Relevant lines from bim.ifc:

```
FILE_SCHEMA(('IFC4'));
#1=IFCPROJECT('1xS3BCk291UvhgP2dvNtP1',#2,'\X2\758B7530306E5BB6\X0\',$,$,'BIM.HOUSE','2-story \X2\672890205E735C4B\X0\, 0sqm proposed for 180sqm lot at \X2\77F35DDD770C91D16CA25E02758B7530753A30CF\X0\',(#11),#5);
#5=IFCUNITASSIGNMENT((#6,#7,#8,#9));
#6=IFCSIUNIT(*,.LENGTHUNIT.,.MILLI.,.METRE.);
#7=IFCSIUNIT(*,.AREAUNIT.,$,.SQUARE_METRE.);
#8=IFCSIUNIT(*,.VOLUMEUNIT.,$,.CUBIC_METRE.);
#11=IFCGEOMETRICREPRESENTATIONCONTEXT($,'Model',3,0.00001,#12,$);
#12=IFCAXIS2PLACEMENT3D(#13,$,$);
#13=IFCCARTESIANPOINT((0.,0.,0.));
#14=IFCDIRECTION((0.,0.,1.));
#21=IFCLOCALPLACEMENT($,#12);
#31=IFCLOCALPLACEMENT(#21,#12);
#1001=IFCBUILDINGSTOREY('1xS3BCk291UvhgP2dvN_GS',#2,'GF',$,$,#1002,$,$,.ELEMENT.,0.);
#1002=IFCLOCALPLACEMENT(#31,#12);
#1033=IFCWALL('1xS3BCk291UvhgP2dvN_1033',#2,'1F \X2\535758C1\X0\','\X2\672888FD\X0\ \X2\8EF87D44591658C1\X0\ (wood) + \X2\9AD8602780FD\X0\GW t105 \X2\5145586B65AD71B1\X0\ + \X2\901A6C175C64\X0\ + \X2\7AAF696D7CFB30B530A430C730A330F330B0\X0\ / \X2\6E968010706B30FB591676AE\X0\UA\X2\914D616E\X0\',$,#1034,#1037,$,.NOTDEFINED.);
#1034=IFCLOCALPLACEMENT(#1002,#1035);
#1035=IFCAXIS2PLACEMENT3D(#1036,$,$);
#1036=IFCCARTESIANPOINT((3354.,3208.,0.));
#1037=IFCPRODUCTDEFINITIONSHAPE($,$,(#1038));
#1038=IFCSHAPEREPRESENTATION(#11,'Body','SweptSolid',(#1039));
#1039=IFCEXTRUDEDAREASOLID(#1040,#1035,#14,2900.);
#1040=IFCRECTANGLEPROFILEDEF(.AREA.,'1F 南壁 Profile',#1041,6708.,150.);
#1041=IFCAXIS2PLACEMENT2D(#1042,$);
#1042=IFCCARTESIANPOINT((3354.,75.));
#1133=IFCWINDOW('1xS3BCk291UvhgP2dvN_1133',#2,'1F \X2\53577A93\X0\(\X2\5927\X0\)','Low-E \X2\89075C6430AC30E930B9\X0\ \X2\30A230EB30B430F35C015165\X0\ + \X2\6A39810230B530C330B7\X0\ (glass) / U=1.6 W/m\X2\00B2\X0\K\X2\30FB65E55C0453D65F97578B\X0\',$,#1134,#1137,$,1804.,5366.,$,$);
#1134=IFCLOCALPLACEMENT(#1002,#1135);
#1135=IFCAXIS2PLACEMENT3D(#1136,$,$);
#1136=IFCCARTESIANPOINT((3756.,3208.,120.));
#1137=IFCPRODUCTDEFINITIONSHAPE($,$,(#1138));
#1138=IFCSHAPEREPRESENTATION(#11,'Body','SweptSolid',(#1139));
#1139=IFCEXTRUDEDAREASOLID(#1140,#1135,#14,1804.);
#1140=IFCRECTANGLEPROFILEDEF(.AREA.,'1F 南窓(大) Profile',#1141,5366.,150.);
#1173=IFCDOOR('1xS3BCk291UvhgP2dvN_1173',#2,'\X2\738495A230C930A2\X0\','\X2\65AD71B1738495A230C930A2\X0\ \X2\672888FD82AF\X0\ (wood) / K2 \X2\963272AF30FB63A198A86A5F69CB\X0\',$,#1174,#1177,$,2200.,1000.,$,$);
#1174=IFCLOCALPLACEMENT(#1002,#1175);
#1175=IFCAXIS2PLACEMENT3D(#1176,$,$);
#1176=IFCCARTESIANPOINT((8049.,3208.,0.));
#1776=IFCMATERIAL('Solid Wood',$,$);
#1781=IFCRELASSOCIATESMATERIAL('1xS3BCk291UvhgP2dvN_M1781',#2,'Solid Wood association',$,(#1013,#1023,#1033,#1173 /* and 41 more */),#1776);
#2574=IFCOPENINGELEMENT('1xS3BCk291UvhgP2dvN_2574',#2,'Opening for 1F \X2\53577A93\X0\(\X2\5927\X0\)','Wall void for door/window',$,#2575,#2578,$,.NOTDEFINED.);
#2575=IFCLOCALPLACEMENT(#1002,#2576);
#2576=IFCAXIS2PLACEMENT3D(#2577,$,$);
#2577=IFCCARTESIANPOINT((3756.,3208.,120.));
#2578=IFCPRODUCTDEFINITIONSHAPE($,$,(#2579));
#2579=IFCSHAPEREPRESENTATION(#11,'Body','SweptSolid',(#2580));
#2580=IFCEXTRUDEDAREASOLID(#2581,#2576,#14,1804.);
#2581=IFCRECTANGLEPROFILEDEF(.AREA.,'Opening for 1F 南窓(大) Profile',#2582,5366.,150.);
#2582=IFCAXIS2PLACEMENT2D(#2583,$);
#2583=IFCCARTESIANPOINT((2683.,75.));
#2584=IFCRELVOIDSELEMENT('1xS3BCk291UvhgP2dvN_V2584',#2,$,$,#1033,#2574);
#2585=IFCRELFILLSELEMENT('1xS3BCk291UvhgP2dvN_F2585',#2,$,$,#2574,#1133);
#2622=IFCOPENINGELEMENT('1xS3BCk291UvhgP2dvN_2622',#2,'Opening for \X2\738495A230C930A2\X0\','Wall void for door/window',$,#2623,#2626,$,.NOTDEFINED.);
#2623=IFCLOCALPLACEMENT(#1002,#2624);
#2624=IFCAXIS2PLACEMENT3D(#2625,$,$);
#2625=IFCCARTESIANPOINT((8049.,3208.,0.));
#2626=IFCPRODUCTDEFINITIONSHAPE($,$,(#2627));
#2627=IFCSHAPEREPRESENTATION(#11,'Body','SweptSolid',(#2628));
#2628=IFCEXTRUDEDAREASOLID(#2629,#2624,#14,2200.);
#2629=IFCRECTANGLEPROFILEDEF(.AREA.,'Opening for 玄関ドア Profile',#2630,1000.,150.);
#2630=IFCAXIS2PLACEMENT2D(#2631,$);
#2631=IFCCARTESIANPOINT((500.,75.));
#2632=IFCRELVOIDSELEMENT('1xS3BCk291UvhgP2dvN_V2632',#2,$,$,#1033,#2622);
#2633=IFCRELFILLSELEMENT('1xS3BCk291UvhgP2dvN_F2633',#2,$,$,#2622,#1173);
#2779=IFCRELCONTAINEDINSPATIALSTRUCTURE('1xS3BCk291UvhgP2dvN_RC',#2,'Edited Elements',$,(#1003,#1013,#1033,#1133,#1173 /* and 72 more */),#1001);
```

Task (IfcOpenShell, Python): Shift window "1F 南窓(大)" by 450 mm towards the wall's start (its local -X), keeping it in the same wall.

```python
import ifcopenshell
import ifcopenshell.api.geometry
import ifcopenshell.util.placement

model = ifcopenshell.open("bim.ifc")

window = model.by_guid("1xS3BCk291UvhgP2dvN_1133")
opening = window.FillsVoids[0].RelatingOpeningElement
wall = opening.VoidsElements[0].RelatingBuildingElement

wall_matrix = ifcopenshell.util.placement.get_local_placement(wall.ObjectPlacement)
shift = wall_matrix[:3, 0] * -450.0
before = ifcopenshell.util.placement.get_local_placement(window.ObjectPlacement)[:3, 3].copy()

# The window is not placed relative to its opening, so move both.
for product in (opening, window):
    matrix = ifcopenshell.util.placement.get_local_placement(product.ObjectPlacement)
    matrix[:3, 3] += shift
    ifcopenshell.api.geometry.edit_object_placement(model, product=product, matrix=matrix, is_si=False)

after = ifcopenshell.util.placement.get_local_placement(window.ObjectPlacement)[:3, 3]
print("window moved by", (after - before).round(3) + 0.0)

model.write("bim_rev.ifc")
```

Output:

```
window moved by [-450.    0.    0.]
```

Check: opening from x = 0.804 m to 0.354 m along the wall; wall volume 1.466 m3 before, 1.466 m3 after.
